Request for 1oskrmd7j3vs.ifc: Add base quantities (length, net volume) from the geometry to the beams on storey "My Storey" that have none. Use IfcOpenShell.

First a look at what the model holds.

```python
import ifcopenshell
import ifcopenshell.util.element
import ifcopenshell.util.unit

model = ifcopenshell.open("1oskrmd7j3vs.ifc")
print(model.schema)
for unit_type in ("LENGTHUNIT", "AREAUNIT", "VOLUMEUNIT"):
    print(unit_type, ifcopenshell.util.unit.calculate_unit_scale(model, unit_type))
storey = next(s for s in model.by_type("IfcBuildingStorey") if s.Name == "My Storey")
beams = [e for e in ifcopenshell.util.element.get_decomposition(storey) if e.is_a("IfcBeam")]
for e in sorted(beams, key=lambda e: e.id()):
    print(e.id(), e.is_a(), e.Name, list(ifcopenshell.util.element.get_psets(e, qtos_only=True)), sep=" | ")
```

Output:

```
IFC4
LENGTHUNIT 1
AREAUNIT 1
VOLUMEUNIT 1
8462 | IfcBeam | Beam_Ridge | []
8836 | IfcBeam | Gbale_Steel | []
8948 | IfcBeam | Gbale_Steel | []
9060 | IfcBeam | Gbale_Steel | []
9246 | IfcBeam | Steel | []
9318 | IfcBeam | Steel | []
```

```python
import ifcopenshell
import ifcopenshell.api.pset
import ifcopenshell.geom
import ifcopenshell.util.element
import ifcopenshell.util.shape
import ifcopenshell.util.unit

model = ifcopenshell.open("1oskrmd7j3vs.ifc")
unit_scale = ifcopenshell.util.unit.calculate_unit_scale(model)
volume_scale = ifcopenshell.util.unit.calculate_unit_scale(model, "VOLUMEUNIT")
settings = ifcopenshell.geom.settings()

storey = next(s for s in model.by_type("IfcBuildingStorey") if s.Name == "My Storey")
beams = [e for e in ifcopenshell.util.element.get_decomposition(storey) if e.is_a("IfcBeam")]

for e in sorted(beams, key=lambda e: e.id()):
    if ifcopenshell.util.element.get_psets(e, qtos_only=True, should_inherit=False):
        continue
    # Geometry comes back in metres, in the element's own axes.
    shape = ifcopenshell.geom.create_shape(settings, e)
    values = {
        "Length": ifcopenshell.util.shape.get_max_xyz(shape.geometry) / unit_scale,
        "NetVolume": ifcopenshell.util.shape.get_volume(shape.geometry) / volume_scale,
    }
    qto = ifcopenshell.api.pset.add_qto(model, product=e, name="Qto_BeamBaseQuantities")
    ifcopenshell.api.pset.edit_qto(model, qto=qto, properties=values)
    print(e.id(), {k: round(v, 3) for k, v in values.items()})

model.write("1oskrmd7j3vs_rev.ifc")
```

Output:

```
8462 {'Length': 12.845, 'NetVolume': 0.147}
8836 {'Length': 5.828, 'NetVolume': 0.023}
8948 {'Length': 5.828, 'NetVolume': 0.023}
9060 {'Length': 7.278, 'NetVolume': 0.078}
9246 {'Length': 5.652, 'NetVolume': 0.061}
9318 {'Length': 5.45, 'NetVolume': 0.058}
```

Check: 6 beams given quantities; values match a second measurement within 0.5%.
